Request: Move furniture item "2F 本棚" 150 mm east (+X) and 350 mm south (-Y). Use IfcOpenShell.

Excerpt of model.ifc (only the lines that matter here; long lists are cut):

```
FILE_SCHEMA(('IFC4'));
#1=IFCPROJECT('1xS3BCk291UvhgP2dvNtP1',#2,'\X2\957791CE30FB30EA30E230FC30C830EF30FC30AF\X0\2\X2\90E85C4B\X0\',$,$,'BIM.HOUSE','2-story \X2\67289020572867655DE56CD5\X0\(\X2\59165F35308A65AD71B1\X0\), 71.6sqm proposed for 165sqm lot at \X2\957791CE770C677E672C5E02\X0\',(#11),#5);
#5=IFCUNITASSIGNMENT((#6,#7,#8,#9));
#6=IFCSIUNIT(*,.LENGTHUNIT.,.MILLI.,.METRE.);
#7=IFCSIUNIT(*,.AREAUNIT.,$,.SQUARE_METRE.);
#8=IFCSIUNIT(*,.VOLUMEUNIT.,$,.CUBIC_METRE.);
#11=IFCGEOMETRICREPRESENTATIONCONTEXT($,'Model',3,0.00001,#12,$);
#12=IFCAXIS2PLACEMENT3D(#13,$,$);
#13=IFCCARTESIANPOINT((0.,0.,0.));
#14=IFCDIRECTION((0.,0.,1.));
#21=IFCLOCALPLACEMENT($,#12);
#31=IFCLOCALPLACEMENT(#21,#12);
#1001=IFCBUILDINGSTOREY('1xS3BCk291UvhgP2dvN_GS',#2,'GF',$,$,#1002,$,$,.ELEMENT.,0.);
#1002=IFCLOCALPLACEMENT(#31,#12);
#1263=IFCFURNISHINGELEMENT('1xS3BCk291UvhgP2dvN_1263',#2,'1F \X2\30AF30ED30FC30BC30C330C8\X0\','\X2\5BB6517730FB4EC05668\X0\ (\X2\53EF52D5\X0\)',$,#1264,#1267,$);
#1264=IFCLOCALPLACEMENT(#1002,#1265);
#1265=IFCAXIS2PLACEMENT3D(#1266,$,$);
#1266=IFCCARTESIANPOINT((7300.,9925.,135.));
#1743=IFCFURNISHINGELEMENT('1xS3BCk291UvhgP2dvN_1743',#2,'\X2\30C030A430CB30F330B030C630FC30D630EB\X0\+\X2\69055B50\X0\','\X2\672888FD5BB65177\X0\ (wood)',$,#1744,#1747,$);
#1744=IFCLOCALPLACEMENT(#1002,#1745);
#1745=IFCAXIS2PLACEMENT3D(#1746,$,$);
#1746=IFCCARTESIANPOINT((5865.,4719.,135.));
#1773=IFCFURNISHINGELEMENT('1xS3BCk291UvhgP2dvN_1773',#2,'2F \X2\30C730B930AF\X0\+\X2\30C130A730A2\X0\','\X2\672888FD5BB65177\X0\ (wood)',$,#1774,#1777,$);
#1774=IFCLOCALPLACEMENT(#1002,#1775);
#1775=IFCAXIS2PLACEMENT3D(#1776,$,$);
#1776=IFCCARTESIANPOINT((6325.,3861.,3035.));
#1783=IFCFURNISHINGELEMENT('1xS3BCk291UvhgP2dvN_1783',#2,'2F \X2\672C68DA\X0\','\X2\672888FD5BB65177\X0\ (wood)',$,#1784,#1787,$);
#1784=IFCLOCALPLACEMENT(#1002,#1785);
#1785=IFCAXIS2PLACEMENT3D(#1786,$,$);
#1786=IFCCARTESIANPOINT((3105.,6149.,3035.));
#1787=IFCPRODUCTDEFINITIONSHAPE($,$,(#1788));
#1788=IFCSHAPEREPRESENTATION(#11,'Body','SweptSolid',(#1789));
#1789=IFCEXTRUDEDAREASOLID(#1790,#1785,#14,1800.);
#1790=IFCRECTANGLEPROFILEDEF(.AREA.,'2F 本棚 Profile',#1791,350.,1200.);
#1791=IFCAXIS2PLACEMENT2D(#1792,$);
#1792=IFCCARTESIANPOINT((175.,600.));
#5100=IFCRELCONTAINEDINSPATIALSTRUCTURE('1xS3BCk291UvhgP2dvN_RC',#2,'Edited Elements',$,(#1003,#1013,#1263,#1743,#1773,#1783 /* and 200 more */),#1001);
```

```python
import ifcopenshell
import ifcopenshell.api.geometry
import ifcopenshell.util.placement
import ifcopenshell.util.unit

model = ifcopenshell.open("model.ifc")
unit_scale = ifcopenshell.util.unit.calculate_unit_scale(model)

item = model.by_guid("1xS3BCk291UvhgP2dvN_1783")
matrix = ifcopenshell.util.placement.get_local_placement(item.ObjectPlacement)
matrix[0, 3] += 0.15 / unit_scale
matrix[1, 3] -= 0.35 / unit_scale
ifcopenshell.api.geometry.edit_object_placement(model, product=item, matrix=matrix, is_si=False)

print(ifcopenshell.util.placement.get_local_placement(item.ObjectPlacement).round(3) + 0.0)

model.write("model_rev.ifc")
```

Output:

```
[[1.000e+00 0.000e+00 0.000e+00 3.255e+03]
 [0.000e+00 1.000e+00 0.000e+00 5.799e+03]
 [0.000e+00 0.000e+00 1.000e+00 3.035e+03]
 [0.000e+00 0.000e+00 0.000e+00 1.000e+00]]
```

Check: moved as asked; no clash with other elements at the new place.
